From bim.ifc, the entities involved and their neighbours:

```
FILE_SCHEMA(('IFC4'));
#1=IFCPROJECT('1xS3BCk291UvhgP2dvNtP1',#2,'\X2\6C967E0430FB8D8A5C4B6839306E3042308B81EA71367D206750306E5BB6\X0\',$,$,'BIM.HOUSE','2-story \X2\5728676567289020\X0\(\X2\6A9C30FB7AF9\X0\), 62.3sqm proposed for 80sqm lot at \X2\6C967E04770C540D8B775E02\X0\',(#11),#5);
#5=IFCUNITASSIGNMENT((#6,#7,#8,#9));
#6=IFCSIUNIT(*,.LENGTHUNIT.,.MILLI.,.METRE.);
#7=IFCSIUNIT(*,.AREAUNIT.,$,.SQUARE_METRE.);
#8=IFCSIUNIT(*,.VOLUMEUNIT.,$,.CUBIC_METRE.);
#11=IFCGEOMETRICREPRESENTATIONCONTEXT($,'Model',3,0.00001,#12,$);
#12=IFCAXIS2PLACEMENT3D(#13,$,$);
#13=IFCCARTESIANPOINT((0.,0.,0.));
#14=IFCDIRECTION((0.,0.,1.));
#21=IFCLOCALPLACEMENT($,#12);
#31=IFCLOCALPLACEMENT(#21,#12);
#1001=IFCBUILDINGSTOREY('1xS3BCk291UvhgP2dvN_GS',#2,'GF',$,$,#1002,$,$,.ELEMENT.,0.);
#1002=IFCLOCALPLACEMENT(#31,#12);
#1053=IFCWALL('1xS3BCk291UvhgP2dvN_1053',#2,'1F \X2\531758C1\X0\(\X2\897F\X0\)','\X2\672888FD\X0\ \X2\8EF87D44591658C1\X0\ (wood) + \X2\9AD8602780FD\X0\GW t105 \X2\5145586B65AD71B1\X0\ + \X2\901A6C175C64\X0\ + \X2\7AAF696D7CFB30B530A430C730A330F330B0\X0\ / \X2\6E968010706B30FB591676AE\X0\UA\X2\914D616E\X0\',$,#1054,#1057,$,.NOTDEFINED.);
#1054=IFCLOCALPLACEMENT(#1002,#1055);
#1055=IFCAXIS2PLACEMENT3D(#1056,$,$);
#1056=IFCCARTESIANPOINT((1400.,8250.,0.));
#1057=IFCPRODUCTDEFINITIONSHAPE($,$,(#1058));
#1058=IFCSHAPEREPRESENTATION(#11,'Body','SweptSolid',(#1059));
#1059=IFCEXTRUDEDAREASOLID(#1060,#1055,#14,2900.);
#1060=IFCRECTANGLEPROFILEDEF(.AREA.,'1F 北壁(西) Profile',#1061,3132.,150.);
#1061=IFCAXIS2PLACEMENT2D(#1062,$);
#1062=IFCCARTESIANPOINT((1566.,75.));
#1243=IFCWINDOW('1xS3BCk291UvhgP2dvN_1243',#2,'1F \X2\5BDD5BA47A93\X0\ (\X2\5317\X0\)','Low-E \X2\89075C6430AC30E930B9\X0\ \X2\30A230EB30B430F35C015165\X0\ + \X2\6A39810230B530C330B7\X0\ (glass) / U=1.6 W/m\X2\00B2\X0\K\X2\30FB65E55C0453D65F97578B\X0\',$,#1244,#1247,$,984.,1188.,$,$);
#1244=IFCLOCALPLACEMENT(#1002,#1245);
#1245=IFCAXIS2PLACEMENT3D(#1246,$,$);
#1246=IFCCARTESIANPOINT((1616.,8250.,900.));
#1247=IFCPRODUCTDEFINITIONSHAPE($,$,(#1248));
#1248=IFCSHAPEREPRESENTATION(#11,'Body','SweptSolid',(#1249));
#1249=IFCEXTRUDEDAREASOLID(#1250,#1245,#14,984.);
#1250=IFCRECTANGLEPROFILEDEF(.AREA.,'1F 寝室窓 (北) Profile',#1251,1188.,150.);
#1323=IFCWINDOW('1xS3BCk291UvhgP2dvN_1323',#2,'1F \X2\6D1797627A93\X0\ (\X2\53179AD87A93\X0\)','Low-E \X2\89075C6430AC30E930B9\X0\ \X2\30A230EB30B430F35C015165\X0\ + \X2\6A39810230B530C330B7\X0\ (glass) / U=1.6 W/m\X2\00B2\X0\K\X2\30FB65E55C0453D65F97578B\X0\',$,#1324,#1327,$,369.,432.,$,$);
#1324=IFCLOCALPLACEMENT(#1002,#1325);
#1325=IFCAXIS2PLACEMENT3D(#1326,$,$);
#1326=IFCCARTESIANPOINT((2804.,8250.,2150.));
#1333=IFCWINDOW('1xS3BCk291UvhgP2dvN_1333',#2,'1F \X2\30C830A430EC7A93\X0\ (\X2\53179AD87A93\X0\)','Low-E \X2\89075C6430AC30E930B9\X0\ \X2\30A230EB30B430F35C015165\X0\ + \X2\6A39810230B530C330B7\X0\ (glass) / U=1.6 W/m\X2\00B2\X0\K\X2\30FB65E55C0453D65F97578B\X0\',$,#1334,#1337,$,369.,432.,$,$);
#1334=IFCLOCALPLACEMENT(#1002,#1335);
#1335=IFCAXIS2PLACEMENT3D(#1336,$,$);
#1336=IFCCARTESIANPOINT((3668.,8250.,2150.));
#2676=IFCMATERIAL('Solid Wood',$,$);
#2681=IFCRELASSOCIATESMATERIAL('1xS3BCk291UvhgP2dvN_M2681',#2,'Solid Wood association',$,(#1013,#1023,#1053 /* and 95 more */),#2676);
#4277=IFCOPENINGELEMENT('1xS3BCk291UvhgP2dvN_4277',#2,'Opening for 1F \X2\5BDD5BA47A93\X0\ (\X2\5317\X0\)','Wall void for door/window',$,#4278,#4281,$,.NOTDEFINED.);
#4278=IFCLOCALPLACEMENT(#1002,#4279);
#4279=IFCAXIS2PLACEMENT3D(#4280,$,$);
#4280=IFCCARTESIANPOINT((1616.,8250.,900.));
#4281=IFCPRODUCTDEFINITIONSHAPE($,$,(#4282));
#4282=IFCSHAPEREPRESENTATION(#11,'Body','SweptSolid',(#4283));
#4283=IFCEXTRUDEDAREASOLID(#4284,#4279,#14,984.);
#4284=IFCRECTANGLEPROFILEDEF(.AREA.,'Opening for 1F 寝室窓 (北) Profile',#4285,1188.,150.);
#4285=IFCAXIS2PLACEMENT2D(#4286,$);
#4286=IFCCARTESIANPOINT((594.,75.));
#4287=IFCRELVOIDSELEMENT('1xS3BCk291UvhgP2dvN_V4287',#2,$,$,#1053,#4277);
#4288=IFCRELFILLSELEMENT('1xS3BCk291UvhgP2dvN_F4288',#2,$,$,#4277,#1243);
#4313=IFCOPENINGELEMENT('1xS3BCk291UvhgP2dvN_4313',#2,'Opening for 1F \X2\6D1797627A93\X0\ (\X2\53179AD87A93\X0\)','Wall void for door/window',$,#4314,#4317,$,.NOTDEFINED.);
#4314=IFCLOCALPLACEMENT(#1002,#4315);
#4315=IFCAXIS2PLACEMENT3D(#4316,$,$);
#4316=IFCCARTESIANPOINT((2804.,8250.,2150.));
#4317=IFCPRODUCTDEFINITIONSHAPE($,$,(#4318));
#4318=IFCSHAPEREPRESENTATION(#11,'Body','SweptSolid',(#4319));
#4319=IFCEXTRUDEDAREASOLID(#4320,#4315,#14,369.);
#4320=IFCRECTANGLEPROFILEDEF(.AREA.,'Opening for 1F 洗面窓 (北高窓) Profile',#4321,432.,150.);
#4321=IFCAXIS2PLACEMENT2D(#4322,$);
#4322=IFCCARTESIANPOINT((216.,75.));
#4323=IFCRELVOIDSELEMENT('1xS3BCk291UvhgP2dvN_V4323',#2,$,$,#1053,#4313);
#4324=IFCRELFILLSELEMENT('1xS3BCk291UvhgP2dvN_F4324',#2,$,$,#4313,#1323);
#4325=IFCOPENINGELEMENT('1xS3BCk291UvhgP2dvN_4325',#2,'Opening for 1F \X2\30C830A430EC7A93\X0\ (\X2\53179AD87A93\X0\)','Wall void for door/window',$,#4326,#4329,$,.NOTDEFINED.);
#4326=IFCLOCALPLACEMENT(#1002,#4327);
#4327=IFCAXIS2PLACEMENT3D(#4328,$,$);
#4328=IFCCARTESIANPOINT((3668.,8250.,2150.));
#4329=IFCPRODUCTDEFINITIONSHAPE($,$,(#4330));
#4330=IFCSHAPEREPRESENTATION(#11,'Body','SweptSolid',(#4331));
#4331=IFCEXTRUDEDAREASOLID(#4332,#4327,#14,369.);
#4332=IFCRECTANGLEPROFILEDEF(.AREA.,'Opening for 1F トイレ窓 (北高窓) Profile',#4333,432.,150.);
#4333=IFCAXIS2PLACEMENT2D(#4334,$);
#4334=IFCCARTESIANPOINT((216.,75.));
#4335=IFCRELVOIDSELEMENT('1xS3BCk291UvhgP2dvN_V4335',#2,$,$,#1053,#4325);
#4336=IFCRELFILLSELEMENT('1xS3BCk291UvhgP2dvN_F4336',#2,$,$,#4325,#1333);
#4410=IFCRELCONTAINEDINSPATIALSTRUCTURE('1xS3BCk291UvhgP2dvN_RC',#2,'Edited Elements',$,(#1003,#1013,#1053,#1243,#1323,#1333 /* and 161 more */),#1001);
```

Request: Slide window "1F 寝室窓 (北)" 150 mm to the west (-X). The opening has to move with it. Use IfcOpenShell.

```python
import ifcopenshell
import ifcopenshell.api.geometry
import ifcopenshell.util.placement

model = ifcopenshell.open("bim.ifc")

window = model.by_guid("1xS3BCk291UvhgP2dvN_1243")
opening = window.FillsVoids[0].RelatingOpeningElement
wall = opening.VoidsElements[0].RelatingBuildingElement

wall_matrix = ifcopenshell.util.placement.get_local_placement(wall.ObjectPlacement)
shift = wall_matrix[:3, 0] * -150.0
before = ifcopenshell.util.placement.get_local_placement(window.ObjectPlacement)[:3, 3].copy()

# The window is not placed relative to its opening, so move both.
for product in (opening, window):
    matrix = ifcopenshell.util.placement.get_local_placement(product.ObjectPlacement)
    matrix[:3, 3] += shift
    ifcopenshell.api.geometry.edit_object_placement(model, product=product, matrix=matrix, is_si=False)

after = ifcopenshell.util.placement.get_local_placement(window.ObjectPlacement)[:3, 3]
print("window moved by", (after - before).round(3) + 0.0)

model.write("bim_rev.ifc")
```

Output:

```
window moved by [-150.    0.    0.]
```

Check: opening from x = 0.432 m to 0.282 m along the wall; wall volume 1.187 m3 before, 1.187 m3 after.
